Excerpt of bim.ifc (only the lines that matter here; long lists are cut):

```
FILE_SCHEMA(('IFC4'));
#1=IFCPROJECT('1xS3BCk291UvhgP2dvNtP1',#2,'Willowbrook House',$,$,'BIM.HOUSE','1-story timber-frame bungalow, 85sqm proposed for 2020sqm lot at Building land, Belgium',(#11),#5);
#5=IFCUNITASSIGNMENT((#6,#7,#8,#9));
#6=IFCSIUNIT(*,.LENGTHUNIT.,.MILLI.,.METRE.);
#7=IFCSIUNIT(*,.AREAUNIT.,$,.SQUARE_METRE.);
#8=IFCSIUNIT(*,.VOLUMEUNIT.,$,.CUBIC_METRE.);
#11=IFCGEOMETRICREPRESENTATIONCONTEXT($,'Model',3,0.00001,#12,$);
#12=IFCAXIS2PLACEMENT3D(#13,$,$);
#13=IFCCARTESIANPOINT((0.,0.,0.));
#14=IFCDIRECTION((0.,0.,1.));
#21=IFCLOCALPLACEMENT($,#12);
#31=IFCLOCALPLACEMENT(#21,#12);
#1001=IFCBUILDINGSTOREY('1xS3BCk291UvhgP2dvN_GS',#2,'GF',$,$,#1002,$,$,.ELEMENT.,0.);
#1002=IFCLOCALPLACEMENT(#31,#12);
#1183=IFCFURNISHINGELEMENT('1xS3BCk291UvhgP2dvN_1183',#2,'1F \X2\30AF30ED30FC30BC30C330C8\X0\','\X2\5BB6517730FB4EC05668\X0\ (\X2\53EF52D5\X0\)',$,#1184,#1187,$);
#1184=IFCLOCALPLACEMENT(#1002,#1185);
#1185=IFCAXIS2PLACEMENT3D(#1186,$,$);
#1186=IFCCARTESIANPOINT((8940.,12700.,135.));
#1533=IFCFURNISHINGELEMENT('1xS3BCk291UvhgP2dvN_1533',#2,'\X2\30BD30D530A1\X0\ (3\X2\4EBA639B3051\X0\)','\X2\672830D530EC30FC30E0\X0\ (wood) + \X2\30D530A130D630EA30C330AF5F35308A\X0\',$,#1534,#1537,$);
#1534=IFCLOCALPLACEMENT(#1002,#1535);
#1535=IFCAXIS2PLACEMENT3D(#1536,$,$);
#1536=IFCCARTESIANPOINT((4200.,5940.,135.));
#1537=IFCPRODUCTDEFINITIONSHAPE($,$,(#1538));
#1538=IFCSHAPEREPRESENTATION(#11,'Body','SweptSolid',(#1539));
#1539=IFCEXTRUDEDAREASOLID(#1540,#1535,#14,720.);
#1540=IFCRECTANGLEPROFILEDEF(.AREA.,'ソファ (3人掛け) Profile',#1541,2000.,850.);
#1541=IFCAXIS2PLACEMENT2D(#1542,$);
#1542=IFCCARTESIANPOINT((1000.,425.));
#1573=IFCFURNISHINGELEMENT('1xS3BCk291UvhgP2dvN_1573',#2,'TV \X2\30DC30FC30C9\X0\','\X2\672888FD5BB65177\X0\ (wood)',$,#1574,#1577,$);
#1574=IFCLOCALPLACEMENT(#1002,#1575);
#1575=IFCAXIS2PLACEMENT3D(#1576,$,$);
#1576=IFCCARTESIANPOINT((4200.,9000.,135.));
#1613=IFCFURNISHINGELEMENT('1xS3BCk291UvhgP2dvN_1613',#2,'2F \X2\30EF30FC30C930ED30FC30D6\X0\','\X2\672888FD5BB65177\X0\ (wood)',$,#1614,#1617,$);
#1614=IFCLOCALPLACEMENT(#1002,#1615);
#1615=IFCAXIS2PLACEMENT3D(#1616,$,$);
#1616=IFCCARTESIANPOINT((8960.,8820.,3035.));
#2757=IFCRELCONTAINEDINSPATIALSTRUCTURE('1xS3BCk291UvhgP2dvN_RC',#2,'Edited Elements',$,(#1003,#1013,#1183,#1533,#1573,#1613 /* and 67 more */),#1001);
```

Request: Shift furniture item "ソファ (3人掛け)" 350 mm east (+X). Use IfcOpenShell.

```python
import ifcopenshell
import ifcopenshell.api.geometry
import ifcopenshell.util.placement
import ifcopenshell.util.unit

model = ifcopenshell.open("bim.ifc")
unit_scale = ifcopenshell.util.unit.calculate_unit_scale(model)

item = model.by_guid("1xS3BCk291UvhgP2dvN_1533")
matrix = ifcopenshell.util.placement.get_local_placement(item.ObjectPlacement)
matrix[0, 3] += 0.35 / unit_scale
ifcopenshell.api.geometry.edit_object_placement(model, product=item, matrix=matrix, is_si=False)

print(ifcopenshell.util.placement.get_local_placement(item.ObjectPlacement).round(3) + 0.0)

model.write("bim_v2.ifc")
```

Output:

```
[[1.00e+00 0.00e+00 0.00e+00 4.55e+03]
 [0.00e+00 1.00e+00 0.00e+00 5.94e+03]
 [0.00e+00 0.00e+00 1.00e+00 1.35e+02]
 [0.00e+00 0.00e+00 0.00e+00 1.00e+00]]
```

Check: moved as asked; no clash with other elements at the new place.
